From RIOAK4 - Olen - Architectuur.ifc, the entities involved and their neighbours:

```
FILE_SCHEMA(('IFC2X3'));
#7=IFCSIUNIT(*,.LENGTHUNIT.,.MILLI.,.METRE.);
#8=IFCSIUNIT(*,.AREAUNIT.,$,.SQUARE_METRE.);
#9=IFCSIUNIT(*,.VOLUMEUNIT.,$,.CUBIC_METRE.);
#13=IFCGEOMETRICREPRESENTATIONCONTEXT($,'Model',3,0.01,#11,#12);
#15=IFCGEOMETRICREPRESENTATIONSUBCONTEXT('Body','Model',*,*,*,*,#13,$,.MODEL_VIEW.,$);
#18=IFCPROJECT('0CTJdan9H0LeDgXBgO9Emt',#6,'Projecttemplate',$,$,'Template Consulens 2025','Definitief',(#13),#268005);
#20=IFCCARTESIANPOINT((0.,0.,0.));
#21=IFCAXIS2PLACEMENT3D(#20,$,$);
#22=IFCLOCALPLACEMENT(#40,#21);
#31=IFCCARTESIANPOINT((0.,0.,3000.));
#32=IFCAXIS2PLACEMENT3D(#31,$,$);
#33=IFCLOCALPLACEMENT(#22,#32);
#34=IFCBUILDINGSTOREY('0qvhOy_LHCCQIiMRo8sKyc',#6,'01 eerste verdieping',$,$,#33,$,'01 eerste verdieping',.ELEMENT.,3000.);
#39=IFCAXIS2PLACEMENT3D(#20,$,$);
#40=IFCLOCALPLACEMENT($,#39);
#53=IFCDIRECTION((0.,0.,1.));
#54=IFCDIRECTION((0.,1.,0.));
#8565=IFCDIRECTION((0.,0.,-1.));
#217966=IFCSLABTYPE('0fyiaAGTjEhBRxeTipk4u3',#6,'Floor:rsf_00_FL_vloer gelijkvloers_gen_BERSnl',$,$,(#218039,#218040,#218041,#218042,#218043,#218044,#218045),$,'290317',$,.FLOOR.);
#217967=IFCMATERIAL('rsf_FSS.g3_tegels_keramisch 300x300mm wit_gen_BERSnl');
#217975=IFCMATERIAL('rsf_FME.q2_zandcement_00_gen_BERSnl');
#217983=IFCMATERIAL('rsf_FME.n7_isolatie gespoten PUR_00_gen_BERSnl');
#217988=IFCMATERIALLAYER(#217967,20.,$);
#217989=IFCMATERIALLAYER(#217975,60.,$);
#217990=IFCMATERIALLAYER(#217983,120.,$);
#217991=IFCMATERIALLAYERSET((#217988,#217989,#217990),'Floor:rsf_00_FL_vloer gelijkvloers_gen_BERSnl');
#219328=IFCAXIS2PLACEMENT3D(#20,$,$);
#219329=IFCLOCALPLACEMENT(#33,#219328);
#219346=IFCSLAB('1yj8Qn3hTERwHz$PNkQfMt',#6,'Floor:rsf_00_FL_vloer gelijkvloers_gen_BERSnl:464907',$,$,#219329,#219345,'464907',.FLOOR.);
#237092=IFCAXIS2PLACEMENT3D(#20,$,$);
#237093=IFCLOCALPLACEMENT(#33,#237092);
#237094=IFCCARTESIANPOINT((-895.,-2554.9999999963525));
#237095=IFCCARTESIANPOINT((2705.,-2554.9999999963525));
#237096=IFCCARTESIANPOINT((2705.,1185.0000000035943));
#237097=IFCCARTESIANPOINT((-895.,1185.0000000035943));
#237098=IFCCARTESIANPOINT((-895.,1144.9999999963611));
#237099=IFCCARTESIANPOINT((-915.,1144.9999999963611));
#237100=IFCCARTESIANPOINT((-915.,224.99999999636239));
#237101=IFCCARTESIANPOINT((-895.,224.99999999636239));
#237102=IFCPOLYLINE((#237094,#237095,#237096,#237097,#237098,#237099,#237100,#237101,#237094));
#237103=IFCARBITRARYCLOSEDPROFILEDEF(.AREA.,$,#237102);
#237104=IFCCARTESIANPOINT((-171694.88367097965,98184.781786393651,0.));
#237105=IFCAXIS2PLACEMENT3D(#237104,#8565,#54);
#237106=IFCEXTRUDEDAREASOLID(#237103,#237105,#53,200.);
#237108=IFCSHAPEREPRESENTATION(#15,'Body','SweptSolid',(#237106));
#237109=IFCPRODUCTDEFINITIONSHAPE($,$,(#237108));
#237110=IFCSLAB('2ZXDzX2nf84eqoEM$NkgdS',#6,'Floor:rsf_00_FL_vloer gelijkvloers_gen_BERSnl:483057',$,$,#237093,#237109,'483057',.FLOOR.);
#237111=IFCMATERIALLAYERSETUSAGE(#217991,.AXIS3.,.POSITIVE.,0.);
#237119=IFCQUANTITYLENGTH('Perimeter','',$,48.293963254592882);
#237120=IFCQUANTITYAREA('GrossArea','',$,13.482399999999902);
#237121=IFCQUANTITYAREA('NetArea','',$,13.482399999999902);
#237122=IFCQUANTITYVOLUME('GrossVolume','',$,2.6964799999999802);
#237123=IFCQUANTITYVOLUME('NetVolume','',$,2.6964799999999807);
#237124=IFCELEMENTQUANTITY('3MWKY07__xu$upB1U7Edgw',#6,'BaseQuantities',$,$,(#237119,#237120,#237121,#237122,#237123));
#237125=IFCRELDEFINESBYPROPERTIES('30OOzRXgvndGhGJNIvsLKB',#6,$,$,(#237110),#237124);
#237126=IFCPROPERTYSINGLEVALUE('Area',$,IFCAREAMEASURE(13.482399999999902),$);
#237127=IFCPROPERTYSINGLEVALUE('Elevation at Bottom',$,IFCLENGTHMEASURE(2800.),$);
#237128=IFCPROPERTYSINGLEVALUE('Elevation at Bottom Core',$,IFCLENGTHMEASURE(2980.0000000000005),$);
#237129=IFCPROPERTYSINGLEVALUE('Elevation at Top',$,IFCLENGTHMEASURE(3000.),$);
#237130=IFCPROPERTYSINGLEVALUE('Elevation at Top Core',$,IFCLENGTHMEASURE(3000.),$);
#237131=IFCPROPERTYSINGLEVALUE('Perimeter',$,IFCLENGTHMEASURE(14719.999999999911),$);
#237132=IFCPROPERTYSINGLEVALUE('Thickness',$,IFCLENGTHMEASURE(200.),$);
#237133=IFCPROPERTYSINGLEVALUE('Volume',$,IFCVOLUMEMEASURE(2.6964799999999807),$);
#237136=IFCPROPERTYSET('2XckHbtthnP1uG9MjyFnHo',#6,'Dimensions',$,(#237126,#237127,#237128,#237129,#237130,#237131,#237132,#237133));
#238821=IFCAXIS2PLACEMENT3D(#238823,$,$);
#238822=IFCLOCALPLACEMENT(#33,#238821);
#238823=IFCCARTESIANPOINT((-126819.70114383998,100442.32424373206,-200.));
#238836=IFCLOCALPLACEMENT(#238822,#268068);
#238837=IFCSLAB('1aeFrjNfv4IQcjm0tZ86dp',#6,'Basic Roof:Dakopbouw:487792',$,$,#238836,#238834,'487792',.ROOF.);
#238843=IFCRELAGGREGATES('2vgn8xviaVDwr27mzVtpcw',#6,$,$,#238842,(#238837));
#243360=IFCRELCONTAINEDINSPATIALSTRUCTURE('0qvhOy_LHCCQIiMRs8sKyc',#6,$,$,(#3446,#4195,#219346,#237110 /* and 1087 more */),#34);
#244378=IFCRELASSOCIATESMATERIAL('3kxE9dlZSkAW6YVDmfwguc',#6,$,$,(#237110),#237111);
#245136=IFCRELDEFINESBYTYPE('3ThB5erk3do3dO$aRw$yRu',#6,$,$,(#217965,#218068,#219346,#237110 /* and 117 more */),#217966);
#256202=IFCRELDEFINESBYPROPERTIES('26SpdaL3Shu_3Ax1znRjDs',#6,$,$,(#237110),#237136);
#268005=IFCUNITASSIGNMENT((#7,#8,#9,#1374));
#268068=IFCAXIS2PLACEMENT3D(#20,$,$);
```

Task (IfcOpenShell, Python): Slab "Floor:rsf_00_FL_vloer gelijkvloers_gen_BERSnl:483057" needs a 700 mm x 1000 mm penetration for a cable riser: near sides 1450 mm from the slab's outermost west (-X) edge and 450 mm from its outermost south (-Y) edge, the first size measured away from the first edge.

```python
import numpy as np
import ifcopenshell
import ifcopenshell.api.feature
import ifcopenshell.api.geometry
import ifcopenshell.api.pset
import ifcopenshell.api.root
import ifcopenshell.geom
import ifcopenshell.util.element
import ifcopenshell.util.placement
import ifcopenshell.util.representation
import ifcopenshell.util.shape
import ifcopenshell.util.unit

model = ifcopenshell.open("RIOAK4 - Olen - Architectuur.ifc")
unit_scale = ifcopenshell.util.unit.calculate_unit_scale(model)
area_scale = ifcopenshell.util.unit.calculate_unit_scale(model, "AREAUNIT")
volume_scale = ifcopenshell.util.unit.calculate_unit_scale(model, "VOLUMEUNIT")
settings = ifcopenshell.geom.settings()


def volume(element):
    """Net volume in cubic metres, openings subtracted."""
    shape = ifcopenshell.geom.create_shape(settings, element)
    return ifcopenshell.util.shape.get_volume(shape.geometry)


slab = model.by_id(237110)
before = volume(slab)

# Extent in the slab's own axes, in metres. The edges named are its -X and -Y sides.
slab_shape = ifcopenshell.geom.create_shape(settings, slab)
vertices = ifcopenshell.util.shape.get_vertices(slab_shape.geometry)
x_min, y_min, bottom = vertices.min(axis=0)
top = vertices[:, 2].max()

opening = ifcopenshell.api.root.create_entity(model, ifc_class="IfcOpeningElement", name="Cable riser opening")
context = ifcopenshell.util.representation.get_context(model, "Model", "Body", "MODEL_VIEW")
width, depth = 0.7, 1
outline = [(0.0, 0.0), (width, 0.0), (width, depth), (0.0, depth), (0.0, 0.0)]
# Overshoot both faces by 50 mm so the cut is clean.
shape = ifcopenshell.api.geometry.add_slab_representation(
    model, context=context, depth=top - bottom + 0.1, polyline=outline
)
ifcopenshell.api.geometry.assign_representation(model, product=opening, representation=shape)

matrix = ifcopenshell.util.placement.get_local_placement(slab.ObjectPlacement)
matrix[:, 3] = matrix @ np.append(np.array([x_min + 1.45, y_min + 0.45, bottom - 0.05]) / unit_scale, 1.0)
ifcopenshell.api.geometry.edit_object_placement(model, product=opening, matrix=matrix, is_si=False)
ifcopenshell.api.feature.add_feature(model, feature=opening, element=slab)

after = volume(slab)

# Update the slab's stored quantities.
qto = model.by_id(ifcopenshell.util.element.get_pset(slab, "BaseQuantities", should_inherit=False)["id"])
ifcopenshell.api.pset.edit_qto(model, qto=qto, properties={
    "NetArea": after / (top - bottom) / area_scale,
    "NetVolume": after / volume_scale,
})
pset = model.by_id(ifcopenshell.util.element.get_pset(slab, "Dimensions", should_inherit=False)["id"])
ifcopenshell.api.pset.edit_pset(model, pset=pset, properties={
    "Area": model.create_entity("IfcAreaMeasure", after / (top - bottom) / area_scale),
    "Volume": model.create_entity("IfcVolumeMeasure", after / volume_scale),
})

print(f"slab volume {before:.3f} -> {after:.3f} m3")

model.write("RIOAK4 - Olen - Architectuur_updated.ifc")
```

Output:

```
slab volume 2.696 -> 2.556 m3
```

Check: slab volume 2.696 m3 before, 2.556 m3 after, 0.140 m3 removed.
